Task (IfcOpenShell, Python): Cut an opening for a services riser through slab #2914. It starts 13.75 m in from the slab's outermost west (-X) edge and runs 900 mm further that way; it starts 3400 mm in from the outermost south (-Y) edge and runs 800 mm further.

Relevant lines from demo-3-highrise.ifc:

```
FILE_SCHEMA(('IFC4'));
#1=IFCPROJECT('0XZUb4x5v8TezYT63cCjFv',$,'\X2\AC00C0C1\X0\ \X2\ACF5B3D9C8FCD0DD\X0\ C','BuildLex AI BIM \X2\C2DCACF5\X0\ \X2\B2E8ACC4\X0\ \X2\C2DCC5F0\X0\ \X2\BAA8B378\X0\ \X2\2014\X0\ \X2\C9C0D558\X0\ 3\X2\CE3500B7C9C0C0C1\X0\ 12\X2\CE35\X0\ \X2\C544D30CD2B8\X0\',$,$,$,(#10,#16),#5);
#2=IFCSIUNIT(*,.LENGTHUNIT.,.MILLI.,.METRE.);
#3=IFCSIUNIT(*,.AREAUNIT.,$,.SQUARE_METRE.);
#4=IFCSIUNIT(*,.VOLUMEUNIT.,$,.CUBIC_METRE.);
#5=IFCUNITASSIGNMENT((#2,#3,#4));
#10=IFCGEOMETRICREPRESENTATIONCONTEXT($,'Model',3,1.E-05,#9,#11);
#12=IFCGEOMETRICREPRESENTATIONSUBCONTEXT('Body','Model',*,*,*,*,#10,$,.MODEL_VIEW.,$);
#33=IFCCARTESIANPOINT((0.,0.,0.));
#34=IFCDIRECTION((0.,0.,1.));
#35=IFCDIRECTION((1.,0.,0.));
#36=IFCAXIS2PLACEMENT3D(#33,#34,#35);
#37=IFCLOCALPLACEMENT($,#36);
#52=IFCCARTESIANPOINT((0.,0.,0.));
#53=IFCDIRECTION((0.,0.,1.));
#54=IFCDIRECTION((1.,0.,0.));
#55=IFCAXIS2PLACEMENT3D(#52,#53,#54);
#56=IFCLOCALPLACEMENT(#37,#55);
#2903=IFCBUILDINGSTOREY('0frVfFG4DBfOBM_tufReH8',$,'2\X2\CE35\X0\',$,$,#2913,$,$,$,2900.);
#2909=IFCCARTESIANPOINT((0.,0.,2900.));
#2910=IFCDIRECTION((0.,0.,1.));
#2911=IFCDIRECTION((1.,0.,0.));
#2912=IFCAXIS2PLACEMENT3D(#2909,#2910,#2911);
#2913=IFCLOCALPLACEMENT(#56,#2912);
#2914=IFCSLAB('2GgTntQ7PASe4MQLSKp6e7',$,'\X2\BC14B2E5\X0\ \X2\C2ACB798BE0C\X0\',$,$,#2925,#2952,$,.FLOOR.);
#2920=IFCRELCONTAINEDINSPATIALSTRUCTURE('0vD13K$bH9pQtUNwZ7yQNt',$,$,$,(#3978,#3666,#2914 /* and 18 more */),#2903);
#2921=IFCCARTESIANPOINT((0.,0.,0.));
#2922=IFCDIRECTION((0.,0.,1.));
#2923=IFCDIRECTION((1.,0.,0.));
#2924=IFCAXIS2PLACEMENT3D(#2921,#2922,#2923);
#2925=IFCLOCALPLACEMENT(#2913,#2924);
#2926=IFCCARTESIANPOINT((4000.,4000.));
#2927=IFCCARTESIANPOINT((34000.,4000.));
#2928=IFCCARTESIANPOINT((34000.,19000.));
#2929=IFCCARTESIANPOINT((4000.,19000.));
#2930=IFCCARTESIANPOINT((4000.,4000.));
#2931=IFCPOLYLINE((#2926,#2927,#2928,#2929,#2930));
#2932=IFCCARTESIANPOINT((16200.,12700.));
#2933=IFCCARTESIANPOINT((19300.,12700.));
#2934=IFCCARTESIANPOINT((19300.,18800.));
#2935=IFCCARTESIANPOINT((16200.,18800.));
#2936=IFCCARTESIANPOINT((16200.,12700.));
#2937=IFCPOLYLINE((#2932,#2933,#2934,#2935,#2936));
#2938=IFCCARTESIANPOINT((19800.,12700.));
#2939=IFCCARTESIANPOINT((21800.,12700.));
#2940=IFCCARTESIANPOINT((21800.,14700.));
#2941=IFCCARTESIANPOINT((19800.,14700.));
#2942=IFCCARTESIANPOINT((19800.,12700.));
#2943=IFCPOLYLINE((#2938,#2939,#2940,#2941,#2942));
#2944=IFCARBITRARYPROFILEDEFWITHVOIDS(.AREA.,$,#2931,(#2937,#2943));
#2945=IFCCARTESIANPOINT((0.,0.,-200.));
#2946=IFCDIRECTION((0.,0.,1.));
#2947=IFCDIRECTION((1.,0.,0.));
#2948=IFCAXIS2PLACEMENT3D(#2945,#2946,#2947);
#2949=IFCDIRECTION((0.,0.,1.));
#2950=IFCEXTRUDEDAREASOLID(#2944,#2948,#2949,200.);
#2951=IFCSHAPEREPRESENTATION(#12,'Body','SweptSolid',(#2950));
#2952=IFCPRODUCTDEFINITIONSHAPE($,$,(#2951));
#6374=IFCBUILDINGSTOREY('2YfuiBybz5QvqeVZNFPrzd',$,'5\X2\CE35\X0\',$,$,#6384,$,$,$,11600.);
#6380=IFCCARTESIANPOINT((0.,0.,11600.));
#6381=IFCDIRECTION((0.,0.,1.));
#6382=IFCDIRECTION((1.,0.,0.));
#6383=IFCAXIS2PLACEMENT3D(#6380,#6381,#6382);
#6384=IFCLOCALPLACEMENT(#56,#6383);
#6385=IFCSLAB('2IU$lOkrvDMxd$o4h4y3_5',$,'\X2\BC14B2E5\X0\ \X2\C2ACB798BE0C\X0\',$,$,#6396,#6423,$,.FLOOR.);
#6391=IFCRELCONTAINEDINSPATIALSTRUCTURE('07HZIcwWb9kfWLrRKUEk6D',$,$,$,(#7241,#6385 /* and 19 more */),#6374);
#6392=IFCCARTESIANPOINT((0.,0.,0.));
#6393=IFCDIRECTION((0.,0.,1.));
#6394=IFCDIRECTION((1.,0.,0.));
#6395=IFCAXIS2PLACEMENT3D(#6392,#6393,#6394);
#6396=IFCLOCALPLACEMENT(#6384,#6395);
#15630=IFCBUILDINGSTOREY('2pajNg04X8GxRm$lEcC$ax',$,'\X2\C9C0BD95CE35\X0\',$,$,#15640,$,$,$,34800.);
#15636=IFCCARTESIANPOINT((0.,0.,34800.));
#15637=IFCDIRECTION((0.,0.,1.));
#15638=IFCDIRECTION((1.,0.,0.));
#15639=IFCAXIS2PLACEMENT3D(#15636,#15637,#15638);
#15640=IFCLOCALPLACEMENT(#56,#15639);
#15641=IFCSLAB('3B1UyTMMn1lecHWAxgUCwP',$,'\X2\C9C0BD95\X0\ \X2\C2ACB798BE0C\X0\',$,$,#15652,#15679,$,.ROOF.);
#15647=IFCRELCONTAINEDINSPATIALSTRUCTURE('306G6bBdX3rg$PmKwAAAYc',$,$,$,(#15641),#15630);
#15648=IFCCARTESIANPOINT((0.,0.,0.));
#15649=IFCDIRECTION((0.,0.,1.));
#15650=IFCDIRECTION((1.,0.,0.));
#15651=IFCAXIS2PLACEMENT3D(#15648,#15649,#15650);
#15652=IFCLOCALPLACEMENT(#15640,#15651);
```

```python
import numpy as np
import ifcopenshell
import ifcopenshell.api.feature
import ifcopenshell.api.geometry
import ifcopenshell.api.root
import ifcopenshell.geom
import ifcopenshell.util.placement
import ifcopenshell.util.representation
import ifcopenshell.util.shape
import ifcopenshell.util.unit

model = ifcopenshell.open("demo-3-highrise.ifc")
unit_scale = ifcopenshell.util.unit.calculate_unit_scale(model)
settings = ifcopenshell.geom.settings()


def volume(element):
    """Net volume in cubic metres, openings subtracted."""
    shape = ifcopenshell.geom.create_shape(settings, element)
    return ifcopenshell.util.shape.get_volume(shape.geometry)


slab = model.by_guid("2GgTntQ7PASe4MQLSKp6e7")
before = volume(slab)

# Extent in the slab's own axes, in metres. The edges named are its -X and -Y sides.
slab_shape = ifcopenshell.geom.create_shape(settings, slab)
vertices = ifcopenshell.util.shape.get_vertices(slab_shape.geometry)
x_min, y_min, bottom = vertices.min(axis=0)
top = vertices[:, 2].max()

opening = ifcopenshell.api.root.create_entity(model, ifc_class="IfcOpeningElement", name="Services riser opening", predefined_type="OPENING")
context = ifcopenshell.util.representation.get_context(model, "Model", "Body", "MODEL_VIEW")
width, depth = 0.9, 0.8
outline = [(0.0, 0.0), (width, 0.0), (width, depth), (0.0, depth), (0.0, 0.0)]
# Overshoot both faces by 50 mm so the cut is clean.
shape = ifcopenshell.api.geometry.add_slab_representation(
    model, context=context, depth=top - bottom + 0.1, polyline=outline
)
ifcopenshell.api.geometry.assign_representation(model, product=opening, representation=shape)

matrix = ifcopenshell.util.placement.get_local_placement(slab.ObjectPlacement)
matrix[:, 3] = matrix @ np.append(np.array([x_min + 13.75, y_min + 3.4, bottom - 0.05]) / unit_scale, 1.0)
ifcopenshell.api.geometry.edit_object_placement(model, product=opening, matrix=matrix, is_si=False)
ifcopenshell.api.feature.add_feature(model, feature=opening, element=slab)

after = volume(slab)

print(f"slab volume {before:.3f} -> {after:.3f} m3")

model.write("demo-3-highrise_updated.ifc")
```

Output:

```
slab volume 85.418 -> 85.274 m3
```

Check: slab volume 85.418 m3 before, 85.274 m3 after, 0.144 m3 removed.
